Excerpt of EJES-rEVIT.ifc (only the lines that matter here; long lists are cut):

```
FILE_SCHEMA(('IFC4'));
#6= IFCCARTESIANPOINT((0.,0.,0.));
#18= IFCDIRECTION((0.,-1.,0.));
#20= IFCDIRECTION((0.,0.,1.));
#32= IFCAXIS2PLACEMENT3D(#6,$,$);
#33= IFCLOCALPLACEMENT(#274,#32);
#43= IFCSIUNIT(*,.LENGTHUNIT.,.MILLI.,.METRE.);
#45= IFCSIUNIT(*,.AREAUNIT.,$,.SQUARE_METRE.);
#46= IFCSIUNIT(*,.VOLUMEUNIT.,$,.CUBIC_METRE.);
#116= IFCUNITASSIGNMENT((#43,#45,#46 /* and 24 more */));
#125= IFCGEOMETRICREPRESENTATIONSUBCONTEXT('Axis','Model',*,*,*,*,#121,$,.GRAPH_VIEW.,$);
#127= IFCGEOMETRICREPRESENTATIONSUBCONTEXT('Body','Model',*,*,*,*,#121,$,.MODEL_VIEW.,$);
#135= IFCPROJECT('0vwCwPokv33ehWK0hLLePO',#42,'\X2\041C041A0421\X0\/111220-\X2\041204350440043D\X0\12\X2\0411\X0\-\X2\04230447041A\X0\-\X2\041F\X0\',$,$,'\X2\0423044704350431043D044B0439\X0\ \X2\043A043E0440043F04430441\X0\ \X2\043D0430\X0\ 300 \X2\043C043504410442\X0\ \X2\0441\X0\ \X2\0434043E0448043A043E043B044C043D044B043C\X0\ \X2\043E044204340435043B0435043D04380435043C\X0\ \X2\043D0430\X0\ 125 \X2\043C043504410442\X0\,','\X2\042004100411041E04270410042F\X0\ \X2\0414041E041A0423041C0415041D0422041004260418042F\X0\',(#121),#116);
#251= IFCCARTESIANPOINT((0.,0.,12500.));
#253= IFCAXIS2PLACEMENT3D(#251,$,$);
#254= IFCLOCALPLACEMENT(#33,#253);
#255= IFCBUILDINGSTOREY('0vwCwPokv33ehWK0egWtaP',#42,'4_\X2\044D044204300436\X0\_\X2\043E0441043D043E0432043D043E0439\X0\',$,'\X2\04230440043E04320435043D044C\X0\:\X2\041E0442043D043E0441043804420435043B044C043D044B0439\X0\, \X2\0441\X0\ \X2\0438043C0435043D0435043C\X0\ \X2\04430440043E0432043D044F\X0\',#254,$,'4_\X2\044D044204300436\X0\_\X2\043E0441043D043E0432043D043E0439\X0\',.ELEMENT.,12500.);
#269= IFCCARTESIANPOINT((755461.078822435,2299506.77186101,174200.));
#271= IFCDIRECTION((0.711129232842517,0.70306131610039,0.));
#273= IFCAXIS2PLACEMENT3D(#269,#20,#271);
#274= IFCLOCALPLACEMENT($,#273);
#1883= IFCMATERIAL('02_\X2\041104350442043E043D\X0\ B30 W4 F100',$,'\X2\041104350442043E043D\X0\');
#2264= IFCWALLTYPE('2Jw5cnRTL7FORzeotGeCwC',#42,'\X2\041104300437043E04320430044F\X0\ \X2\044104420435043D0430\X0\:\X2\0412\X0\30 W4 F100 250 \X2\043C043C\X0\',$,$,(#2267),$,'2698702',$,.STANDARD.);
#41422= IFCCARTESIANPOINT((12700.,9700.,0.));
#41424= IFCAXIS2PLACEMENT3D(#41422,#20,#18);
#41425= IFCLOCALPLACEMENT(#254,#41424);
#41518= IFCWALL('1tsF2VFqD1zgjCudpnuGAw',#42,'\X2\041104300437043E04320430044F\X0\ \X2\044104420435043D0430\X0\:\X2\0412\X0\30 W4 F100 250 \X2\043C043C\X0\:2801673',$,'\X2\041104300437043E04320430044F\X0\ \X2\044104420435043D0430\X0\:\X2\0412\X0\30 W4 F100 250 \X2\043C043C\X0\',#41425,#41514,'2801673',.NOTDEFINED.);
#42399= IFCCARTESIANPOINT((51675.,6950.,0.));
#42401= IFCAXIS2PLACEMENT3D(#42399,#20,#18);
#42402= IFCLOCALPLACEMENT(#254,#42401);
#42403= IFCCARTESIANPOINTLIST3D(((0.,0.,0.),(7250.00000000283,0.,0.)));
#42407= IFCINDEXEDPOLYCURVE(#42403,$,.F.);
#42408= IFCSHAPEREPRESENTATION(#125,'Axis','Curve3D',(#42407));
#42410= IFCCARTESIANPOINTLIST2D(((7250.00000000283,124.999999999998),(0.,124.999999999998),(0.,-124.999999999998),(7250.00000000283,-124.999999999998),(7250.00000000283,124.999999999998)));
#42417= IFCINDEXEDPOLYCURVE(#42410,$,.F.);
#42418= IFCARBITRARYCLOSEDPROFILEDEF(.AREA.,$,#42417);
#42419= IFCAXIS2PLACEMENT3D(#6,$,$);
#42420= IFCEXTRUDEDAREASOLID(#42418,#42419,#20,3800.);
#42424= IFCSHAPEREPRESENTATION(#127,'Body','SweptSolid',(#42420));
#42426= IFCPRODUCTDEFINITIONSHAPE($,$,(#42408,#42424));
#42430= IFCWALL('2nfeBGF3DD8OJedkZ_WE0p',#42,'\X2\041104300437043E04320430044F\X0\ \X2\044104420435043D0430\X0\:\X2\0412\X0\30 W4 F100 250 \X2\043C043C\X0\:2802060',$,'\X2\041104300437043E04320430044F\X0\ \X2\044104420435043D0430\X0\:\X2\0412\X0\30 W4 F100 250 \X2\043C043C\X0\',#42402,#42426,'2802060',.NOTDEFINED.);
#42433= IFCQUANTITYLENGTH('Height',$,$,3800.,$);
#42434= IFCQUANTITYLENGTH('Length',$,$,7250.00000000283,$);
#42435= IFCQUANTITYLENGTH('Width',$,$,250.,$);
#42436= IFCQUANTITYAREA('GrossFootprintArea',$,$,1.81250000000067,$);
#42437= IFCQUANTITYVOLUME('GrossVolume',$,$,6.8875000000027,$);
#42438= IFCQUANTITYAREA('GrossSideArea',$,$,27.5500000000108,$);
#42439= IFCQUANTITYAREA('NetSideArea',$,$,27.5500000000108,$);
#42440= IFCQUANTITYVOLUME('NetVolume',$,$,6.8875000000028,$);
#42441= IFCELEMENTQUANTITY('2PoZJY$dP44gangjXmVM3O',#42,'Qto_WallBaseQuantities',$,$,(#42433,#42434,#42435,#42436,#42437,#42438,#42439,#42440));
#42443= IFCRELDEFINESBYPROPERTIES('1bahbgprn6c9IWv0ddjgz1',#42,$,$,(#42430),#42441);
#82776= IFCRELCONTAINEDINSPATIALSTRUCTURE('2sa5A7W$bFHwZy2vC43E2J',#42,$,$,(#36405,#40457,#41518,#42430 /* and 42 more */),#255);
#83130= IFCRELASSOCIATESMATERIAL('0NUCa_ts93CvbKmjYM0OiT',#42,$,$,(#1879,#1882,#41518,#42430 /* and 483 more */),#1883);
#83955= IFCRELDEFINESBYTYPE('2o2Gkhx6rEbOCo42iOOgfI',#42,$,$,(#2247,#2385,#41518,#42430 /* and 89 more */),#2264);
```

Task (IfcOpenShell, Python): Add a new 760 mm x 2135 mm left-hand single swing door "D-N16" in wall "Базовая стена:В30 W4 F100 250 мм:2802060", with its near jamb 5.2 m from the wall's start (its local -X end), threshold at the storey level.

```python
import numpy as np
import ifcopenshell
import ifcopenshell.api.feature
import ifcopenshell.api.geometry
import ifcopenshell.api.pset
import ifcopenshell.api.root
import ifcopenshell.api.spatial
import ifcopenshell.geom
import ifcopenshell.util.element
import ifcopenshell.util.placement
import ifcopenshell.util.representation
import ifcopenshell.util.shape
import ifcopenshell.util.unit

model = ifcopenshell.open("EJES-rEVIT.ifc")
unit_scale = ifcopenshell.util.unit.calculate_unit_scale(model)
area_scale = ifcopenshell.util.unit.calculate_unit_scale(model, "AREAUNIT")
volume_scale = ifcopenshell.util.unit.calculate_unit_scale(model, "VOLUMEUNIT")
settings = ifcopenshell.geom.settings()


def volume(element):
    """Net volume in cubic metres, openings subtracted."""
    shape = ifcopenshell.geom.create_shape(settings, element)
    return ifcopenshell.util.shape.get_volume(shape.geometry)


wall = model.by_guid("2nfeBGF3DD8OJedkZ_WE0p")
storey = ifcopenshell.util.element.get_container(wall, ifc_class="IfcBuildingStorey")
context = ifcopenshell.util.representation.get_context(model, "Model", "Body", "MODEL_VIEW")
before = volume(wall)

width, height, from_end, sill = 0.76, 2.135, 5.2, 0.0  # metres

# The wall runs along its own X axis, and the end named is its -X end.
wall_shape = ifcopenshell.geom.create_shape(settings, wall)
x, y, z = ifcopenshell.util.shape.get_vertices(wall_shape.geometry).T
start = x.min() + from_end
face, thickness = float(y.min()), float(y.max() - y.min())
wall_matrix = ifcopenshell.util.placement.get_local_placement(wall.ObjectPlacement)
level = ifcopenshell.util.placement.get_local_placement(storey.ObjectPlacement)[2, 3]


def in_wall(x, y):
    """Placement at x, y metres in the wall's axes, at sill height."""
    matrix = wall_matrix.copy()
    matrix[:, 3] = wall_matrix @ np.array([x / unit_scale, y / unit_scale, 0.0, 1.0])
    matrix[2, 3] = level + sill / unit_scale
    return matrix


# Opening: a box that overshoots both wall faces by 50 mm.
opening = ifcopenshell.api.root.create_entity(model, ifc_class="IfcOpeningElement", predefined_type="OPENING")
box = ifcopenshell.api.geometry.add_wall_representation(
    model, context=context, length=width, height=height, thickness=thickness + 0.1
)
ifcopenshell.api.geometry.assign_representation(model, product=opening, representation=box)
ifcopenshell.api.geometry.edit_object_placement(model, product=opening, matrix=in_wall(start, face - 0.05), is_si=False)
ifcopenshell.api.feature.add_feature(model, feature=opening, element=wall)

door = ifcopenshell.api.root.create_entity(model, ifc_class="IfcDoor", name="D-N16", predefined_type="DOOR")
door.OverallWidth, door.OverallHeight = width / unit_scale, height / unit_scale
door.OperationType = "SINGLE_SWING_LEFT"
body = ifcopenshell.api.geometry.add_door_representation(
    model,
    context=context,
    overall_width=door.OverallWidth,
    overall_height=door.OverallHeight,
    operation_type="SINGLE_SWING_LEFT",
    lining_properties={"LiningDepth": thickness / unit_scale, "ThresholdDepth": thickness / unit_scale},
)
ifcopenshell.api.geometry.assign_representation(model, product=door, representation=body)
ifcopenshell.api.spatial.assign_container(model, products=[door], relating_structure=storey)
ifcopenshell.api.feature.add_filling(model, opening=opening, element=door)

# The lining spans the wall, so the door starts at the wall face.
ifcopenshell.api.geometry.edit_object_placement(model, product=door, matrix=in_wall(start, face), is_si=False)

after = volume(wall)

# Update the wall's stored quantities.
qto = model.by_id(ifcopenshell.util.element.get_pset(wall, "Qto_WallBaseQuantities", should_inherit=False)["id"])
ifcopenshell.api.pset.edit_qto(model, qto=qto, properties={
    "NetSideArea": after / thickness / area_scale,
    "NetVolume": after / volume_scale,
})

print(f"wall volume {before:.3f} -> {after:.3f} m3")

model.write("EJES-rEVIT_edited.ifc")
```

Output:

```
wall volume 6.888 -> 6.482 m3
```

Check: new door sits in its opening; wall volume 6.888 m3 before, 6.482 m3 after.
